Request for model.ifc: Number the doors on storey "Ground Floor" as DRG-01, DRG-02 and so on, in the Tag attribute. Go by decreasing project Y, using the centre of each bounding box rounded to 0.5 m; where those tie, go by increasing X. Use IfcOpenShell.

First a look at what the model holds.

```python
import ifcopenshell
import ifcopenshell.util.element
import ifcopenshell.util.placement

model = ifcopenshell.open("model.ifc")
print(model.schema)
storey = next(s for s in model.by_type("IfcBuildingStorey") if s.Name == "Ground Floor")
doors = [e for e in ifcopenshell.util.element.get_decomposition(storey) if e.is_a("IfcDoor")]
for e in sorted(doors, key=lambda e: e.id()):
    origin = ifcopenshell.util.placement.get_local_placement(e.ObjectPlacement)[:3, 3]
    print(e.id(), e.Tag, e.Name, origin.round(2) + 0.0, sep=" | ")
```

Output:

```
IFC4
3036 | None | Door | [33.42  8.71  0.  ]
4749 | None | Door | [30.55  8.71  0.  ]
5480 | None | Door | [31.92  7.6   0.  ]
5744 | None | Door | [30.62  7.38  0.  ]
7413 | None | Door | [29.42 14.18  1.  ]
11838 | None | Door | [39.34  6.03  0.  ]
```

```python
import ifcopenshell
import ifcopenshell.geom
import ifcopenshell.util.element
import ifcopenshell.util.shape

model = ifcopenshell.open("model.ifc")
settings = ifcopenshell.geom.settings()
settings.set("use-world-coords", True)


def centre(element):
    shape = ifcopenshell.geom.create_shape(settings, element)
    return ifcopenshell.util.shape.get_bbox_centroid(shape.geometry)


storey = next(s for s in model.by_type("IfcBuildingStorey") if s.Name == "Ground Floor")
doors = [e for e in ifcopenshell.util.element.get_decomposition(storey) if e.is_a("IfcDoor")]

# Insertion points can sit at a corner or the storey origin, so sort by the geometry (in metres).
centres = {e: centre(e) for e in doors}
doors.sort(key=lambda e: (-round(centres[e][1] / 0.5), centres[e][0]))

for i, e in enumerate(doors, start=1):
    number = f"DRG-{i:02d}"
    e.Tag = number
    print(e.id(), number)

model.write("model_rev.ifc")
```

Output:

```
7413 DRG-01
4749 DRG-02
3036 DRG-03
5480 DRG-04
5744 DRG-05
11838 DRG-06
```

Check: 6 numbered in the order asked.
